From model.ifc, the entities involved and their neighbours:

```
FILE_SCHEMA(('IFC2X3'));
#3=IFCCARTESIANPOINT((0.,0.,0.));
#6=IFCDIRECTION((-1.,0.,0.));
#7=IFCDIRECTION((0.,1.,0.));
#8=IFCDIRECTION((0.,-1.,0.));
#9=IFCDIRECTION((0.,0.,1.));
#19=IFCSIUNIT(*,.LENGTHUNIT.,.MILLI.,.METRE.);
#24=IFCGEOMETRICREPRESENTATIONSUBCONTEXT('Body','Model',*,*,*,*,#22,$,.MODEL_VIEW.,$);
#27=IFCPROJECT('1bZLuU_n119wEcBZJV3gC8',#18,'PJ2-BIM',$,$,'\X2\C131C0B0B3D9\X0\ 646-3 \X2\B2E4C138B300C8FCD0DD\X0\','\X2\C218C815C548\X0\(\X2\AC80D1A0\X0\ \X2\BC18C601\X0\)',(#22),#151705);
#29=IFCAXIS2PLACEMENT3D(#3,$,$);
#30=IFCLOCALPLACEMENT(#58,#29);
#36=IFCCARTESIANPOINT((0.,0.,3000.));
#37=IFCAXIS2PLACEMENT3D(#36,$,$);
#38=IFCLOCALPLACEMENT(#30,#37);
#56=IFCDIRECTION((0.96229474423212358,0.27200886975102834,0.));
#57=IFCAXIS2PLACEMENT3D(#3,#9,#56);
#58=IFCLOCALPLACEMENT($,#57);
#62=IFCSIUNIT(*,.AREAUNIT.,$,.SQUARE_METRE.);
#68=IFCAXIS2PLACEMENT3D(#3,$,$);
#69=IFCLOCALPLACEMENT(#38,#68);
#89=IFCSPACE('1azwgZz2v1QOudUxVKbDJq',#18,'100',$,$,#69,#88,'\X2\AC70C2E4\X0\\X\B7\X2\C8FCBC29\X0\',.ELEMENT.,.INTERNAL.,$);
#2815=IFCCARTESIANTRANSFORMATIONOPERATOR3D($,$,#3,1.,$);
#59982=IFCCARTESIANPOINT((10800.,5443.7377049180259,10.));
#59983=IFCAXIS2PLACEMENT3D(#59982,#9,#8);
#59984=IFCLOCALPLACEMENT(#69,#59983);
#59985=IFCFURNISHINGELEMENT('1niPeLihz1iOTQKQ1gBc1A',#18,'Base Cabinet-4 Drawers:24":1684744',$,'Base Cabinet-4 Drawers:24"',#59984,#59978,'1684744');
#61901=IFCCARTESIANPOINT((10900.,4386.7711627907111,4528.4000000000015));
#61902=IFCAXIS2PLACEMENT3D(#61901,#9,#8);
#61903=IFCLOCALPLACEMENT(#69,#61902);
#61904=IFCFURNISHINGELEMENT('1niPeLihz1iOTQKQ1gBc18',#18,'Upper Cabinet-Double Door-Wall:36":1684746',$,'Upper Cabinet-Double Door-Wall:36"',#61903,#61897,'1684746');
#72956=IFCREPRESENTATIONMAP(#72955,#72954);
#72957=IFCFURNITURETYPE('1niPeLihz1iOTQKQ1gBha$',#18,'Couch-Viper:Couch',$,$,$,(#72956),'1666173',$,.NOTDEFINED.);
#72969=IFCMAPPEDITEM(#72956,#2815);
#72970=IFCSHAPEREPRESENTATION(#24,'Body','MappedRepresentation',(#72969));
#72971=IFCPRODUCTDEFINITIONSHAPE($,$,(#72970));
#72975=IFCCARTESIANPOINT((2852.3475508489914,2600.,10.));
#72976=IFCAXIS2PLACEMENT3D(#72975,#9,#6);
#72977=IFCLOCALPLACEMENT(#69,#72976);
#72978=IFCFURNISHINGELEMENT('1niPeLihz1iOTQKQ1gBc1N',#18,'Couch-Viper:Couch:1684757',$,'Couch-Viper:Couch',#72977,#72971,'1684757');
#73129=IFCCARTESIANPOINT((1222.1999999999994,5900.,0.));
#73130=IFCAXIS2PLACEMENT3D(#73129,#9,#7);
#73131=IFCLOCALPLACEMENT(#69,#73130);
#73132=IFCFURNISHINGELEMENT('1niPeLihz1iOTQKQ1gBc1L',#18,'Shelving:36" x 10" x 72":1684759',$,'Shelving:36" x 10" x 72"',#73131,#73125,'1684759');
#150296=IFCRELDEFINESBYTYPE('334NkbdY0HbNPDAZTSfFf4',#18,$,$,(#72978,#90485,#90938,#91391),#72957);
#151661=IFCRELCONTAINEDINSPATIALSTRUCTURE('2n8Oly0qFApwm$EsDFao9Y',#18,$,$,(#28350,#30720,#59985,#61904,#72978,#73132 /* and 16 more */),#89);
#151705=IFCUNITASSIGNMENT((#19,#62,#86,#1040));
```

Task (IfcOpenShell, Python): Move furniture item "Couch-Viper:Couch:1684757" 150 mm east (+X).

```python
import ifcopenshell
import ifcopenshell.api.geometry
import ifcopenshell.util.placement
import ifcopenshell.util.unit

model = ifcopenshell.open("model.ifc")
unit_scale = ifcopenshell.util.unit.calculate_unit_scale(model)

item = model.by_guid("1niPeLihz1iOTQKQ1gBc1N")
matrix = ifcopenshell.util.placement.get_local_placement(item.ObjectPlacement)
matrix[0, 3] += 0.15 / unit_scale
ifcopenshell.api.geometry.edit_object_placement(model, product=item, matrix=matrix, is_si=False)

print(ifcopenshell.util.placement.get_local_placement(item.ObjectPlacement).round(3) + 0.0)

model.write("model_rev.ifc")
```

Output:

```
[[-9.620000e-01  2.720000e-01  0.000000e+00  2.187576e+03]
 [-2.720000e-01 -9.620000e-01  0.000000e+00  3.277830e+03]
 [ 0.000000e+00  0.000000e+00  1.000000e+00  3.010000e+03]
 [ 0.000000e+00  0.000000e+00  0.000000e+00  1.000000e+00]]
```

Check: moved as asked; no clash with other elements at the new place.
